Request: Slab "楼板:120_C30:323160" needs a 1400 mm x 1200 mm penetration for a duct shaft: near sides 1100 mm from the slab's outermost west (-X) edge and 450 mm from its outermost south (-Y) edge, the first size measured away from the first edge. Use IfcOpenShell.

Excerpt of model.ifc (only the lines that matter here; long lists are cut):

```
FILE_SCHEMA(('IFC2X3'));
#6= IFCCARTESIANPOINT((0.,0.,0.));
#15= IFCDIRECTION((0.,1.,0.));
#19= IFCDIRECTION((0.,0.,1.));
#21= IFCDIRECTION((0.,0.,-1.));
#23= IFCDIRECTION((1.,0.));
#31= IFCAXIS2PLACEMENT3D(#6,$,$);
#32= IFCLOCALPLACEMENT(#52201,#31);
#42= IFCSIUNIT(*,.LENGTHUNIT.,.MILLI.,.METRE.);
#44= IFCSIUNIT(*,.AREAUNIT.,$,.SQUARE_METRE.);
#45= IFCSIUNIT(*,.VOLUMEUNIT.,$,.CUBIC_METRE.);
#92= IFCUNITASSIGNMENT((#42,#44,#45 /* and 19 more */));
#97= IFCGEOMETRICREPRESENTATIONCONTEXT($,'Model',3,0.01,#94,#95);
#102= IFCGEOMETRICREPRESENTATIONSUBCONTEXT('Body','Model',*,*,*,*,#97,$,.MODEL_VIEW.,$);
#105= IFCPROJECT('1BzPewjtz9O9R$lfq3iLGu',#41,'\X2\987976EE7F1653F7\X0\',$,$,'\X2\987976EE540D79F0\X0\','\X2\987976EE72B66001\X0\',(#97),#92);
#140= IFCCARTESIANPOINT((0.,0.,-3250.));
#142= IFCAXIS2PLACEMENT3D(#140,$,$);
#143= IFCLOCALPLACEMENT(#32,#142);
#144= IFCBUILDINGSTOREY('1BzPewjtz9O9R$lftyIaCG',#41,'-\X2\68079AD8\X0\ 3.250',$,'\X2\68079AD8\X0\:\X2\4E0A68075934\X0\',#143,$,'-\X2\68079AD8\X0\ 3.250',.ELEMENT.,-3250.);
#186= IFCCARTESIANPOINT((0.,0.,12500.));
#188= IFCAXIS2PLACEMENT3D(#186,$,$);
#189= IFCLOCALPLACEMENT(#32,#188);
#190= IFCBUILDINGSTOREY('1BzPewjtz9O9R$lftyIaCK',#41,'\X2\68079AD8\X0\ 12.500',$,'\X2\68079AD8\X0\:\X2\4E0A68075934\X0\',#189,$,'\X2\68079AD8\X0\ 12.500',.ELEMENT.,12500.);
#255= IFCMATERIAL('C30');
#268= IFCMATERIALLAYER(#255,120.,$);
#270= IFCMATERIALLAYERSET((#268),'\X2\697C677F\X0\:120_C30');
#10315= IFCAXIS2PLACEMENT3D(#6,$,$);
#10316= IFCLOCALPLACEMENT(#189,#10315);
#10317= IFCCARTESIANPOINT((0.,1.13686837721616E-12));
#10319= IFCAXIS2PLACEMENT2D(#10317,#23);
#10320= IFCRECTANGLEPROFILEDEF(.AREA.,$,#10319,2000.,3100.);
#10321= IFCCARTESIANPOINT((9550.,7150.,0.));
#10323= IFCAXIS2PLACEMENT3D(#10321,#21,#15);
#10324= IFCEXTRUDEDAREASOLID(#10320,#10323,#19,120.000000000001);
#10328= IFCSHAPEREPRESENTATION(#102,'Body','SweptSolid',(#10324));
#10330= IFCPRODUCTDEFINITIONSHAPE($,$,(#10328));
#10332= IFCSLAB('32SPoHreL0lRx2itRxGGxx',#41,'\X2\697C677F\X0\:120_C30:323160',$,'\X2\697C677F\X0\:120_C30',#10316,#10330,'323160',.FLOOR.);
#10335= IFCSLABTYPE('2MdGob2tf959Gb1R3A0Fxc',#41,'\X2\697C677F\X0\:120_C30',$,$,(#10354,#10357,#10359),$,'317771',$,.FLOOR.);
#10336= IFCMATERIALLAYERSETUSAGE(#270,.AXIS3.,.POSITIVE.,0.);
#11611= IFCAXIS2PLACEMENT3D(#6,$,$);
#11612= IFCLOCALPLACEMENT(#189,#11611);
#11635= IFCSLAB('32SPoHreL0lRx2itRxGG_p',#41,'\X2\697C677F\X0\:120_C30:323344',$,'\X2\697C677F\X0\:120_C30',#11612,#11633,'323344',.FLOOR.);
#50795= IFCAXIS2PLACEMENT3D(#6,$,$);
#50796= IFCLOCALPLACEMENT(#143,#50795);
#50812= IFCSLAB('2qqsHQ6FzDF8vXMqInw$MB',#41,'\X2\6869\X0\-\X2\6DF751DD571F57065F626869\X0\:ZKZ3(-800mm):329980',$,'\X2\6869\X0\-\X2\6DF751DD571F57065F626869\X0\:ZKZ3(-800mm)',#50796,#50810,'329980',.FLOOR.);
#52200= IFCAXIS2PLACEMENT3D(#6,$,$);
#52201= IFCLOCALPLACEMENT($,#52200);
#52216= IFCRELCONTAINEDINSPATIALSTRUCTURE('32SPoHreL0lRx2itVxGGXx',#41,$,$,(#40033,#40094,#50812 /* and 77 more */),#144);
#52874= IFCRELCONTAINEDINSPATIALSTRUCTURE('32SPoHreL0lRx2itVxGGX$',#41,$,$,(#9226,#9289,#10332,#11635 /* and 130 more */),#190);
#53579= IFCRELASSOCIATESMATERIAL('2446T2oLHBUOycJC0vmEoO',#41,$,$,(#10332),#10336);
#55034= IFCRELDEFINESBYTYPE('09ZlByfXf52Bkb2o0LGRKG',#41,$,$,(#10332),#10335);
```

```python
import numpy as np
import ifcopenshell
import ifcopenshell.api.feature
import ifcopenshell.api.geometry
import ifcopenshell.api.root
import ifcopenshell.geom
import ifcopenshell.util.placement
import ifcopenshell.util.representation
import ifcopenshell.util.shape
import ifcopenshell.util.unit

model = ifcopenshell.open("model.ifc")
unit_scale = ifcopenshell.util.unit.calculate_unit_scale(model)
settings = ifcopenshell.geom.settings()


def volume(element):
    """Net volume in cubic metres, openings subtracted."""
    shape = ifcopenshell.geom.create_shape(settings, element)
    return ifcopenshell.util.shape.get_volume(shape.geometry)


slab = model.by_guid("32SPoHreL0lRx2itRxGGxx")
before = volume(slab)

# Extent in the slab's own axes, in metres. The edges named are its -X and -Y sides.
slab_shape = ifcopenshell.geom.create_shape(settings, slab)
vertices = ifcopenshell.util.shape.get_vertices(slab_shape.geometry)
x_min, y_min, bottom = vertices.min(axis=0)
top = vertices[:, 2].max()

opening = ifcopenshell.api.root.create_entity(model, ifc_class="IfcOpeningElement", name="Duct shaft opening")
context = ifcopenshell.util.representation.get_context(model, "Model", "Body", "MODEL_VIEW")
width, depth = 1.4, 1.2
outline = [(0.0, 0.0), (width, 0.0), (width, depth), (0.0, depth), (0.0, 0.0)]
# Overshoot both faces by 50 mm so the cut is clean.
shape = ifcopenshell.api.geometry.add_slab_representation(
    model, context=context, depth=top - bottom + 0.1, polyline=outline
)
ifcopenshell.api.geometry.assign_representation(model, product=opening, representation=shape)

matrix = ifcopenshell.util.placement.get_local_placement(slab.ObjectPlacement)
matrix[:, 3] = matrix @ np.append(np.array([x_min + 1.1, y_min + 0.45, bottom - 0.05]) / unit_scale, 1.0)
ifcopenshell.api.geometry.edit_object_placement(model, product=opening, matrix=matrix, is_si=False)
ifcopenshell.api.feature.add_feature(model, feature=opening, element=slab)

after = volume(slab)

print(f"slab volume {before:.3f} -> {after:.3f} m3")

model.write("model_edited.ifc")
```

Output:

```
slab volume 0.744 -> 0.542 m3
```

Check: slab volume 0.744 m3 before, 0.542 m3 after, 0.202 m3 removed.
